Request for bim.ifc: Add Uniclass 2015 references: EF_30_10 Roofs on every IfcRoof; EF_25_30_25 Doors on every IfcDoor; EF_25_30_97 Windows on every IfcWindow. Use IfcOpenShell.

First a look at what the model holds.

```python
import ifcopenshell

model = ifcopenshell.open("bim.ifc")
print(model.schema)
print("classifications:", [c.Name for c in model.by_type("IfcClassification")])
for ifc_class in ("IfcDoor", "IfcRoof", "IfcStair", "IfcWall", "IfcWindow"):
    print(ifc_class, len(model.by_type(ifc_class)))
```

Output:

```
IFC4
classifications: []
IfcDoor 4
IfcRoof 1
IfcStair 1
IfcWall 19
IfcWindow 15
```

```python
import ifcopenshell
import ifcopenshell.api.classification

model = ifcopenshell.open("bim.ifc")

system = ifcopenshell.api.classification.add_classification(model, classification="Uniclass 2015")

codes = {
    "IfcRoof": ("EF_30_10", "Roofs"),
    "IfcDoor": ("EF_25_30_25", "Doors"),
    "IfcWindow": ("EF_25_30_97", "Windows"),
}
for ifc_class, (code, name) in codes.items():
    products = model.by_type(ifc_class)
    ifcopenshell.api.classification.add_reference(
        model, products=products, classification=system, identification=code, name=name
    )
    print(code, len(products))

model.write("bim_edited.ifc")
```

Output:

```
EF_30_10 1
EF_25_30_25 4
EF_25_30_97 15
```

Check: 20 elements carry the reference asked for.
